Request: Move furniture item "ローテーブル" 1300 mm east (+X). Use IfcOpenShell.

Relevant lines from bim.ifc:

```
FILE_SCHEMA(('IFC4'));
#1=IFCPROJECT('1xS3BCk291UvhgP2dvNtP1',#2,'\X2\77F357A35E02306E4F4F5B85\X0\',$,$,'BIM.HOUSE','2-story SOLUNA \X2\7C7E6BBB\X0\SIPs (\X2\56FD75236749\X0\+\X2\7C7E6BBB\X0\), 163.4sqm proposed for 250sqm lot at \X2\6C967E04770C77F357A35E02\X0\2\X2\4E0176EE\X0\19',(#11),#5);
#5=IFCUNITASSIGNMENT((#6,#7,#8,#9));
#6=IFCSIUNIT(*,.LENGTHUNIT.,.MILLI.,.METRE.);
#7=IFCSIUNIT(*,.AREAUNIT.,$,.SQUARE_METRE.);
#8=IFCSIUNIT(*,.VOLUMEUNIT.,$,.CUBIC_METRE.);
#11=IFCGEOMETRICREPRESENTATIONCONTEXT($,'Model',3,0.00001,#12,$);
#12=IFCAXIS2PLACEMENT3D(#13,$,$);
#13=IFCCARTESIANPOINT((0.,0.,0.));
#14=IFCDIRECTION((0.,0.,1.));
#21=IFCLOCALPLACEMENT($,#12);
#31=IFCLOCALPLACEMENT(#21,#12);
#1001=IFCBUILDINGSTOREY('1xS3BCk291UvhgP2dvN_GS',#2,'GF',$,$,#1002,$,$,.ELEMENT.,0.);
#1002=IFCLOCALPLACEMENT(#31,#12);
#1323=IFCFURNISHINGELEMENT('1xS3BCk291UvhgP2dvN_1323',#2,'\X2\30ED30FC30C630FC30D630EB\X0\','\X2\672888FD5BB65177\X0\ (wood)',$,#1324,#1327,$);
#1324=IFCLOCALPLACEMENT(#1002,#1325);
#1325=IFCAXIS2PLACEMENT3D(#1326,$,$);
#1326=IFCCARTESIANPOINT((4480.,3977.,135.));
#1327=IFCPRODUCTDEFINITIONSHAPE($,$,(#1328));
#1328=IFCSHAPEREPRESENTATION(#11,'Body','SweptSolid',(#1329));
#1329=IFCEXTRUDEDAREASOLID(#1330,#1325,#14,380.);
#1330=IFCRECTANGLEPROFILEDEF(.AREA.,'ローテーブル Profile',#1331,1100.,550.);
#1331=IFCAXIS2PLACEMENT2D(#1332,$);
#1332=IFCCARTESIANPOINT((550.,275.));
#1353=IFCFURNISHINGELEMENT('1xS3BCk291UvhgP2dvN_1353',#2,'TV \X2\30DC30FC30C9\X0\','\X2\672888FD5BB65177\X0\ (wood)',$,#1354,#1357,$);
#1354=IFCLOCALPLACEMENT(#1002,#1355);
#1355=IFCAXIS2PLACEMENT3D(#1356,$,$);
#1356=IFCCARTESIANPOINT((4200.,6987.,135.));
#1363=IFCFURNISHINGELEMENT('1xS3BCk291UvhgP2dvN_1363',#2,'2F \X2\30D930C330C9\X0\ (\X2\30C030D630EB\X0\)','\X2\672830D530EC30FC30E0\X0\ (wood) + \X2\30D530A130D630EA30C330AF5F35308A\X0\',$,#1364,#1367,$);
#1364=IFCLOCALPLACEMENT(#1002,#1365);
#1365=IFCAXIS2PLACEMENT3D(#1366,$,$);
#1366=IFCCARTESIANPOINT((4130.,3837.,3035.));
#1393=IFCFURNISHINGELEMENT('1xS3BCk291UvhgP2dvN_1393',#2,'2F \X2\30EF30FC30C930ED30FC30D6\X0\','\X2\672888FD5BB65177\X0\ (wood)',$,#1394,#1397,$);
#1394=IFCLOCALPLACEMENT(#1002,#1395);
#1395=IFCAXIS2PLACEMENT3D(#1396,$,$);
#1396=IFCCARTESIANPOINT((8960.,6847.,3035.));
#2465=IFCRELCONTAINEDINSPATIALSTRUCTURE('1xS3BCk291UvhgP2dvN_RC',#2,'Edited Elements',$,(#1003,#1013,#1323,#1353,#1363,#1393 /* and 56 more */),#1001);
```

```python
import ifcopenshell
import ifcopenshell.api.geometry
import ifcopenshell.util.placement
import ifcopenshell.util.unit

model = ifcopenshell.open("bim.ifc")
unit_scale = ifcopenshell.util.unit.calculate_unit_scale(model)

item = model.by_guid("1xS3BCk291UvhgP2dvN_1323")
matrix = ifcopenshell.util.placement.get_local_placement(item.ObjectPlacement)
matrix[0, 3] += 1.3 / unit_scale
ifcopenshell.api.geometry.edit_object_placement(model, product=item, matrix=matrix, is_si=False)

print(ifcopenshell.util.placement.get_local_placement(item.ObjectPlacement).round(3) + 0.0)

model.write("bim_edited.ifc")
```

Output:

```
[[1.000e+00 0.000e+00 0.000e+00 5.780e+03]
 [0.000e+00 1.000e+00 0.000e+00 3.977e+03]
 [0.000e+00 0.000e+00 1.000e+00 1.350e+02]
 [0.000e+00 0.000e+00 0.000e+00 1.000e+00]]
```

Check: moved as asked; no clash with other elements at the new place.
